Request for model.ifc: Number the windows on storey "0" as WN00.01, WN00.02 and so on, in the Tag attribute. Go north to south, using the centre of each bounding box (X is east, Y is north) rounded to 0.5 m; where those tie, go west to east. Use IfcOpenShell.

First a look at what the model holds.

```python
import ifcopenshell
import ifcopenshell.util.element
import ifcopenshell.util.placement

model = ifcopenshell.open("model.ifc")
print(model.schema)
storey = next(s for s in model.by_type("IfcBuildingStorey") if s.Name == "0")
windows = [e for e in ifcopenshell.util.element.get_decomposition(storey) if e.is_a("IfcWindow")]
for e in sorted(windows, key=lambda e: e.id()):
    origin = ifcopenshell.util.placement.get_local_placement(e.ObjectPlacement)[:3, 3]
    print(e.id(), e.Tag, e.Name, origin.round(2) + 0.0, sep=" | ")
```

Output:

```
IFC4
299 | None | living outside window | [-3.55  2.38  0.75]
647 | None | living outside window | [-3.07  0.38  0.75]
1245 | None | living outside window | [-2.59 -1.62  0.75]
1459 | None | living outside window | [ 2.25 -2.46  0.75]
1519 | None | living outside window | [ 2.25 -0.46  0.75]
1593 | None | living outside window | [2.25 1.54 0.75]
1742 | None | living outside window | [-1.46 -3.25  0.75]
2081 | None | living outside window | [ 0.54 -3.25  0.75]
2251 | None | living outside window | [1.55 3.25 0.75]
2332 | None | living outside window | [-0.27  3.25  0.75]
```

```python
import ifcopenshell
import ifcopenshell.geom
import ifcopenshell.util.element
import ifcopenshell.util.shape

model = ifcopenshell.open("model.ifc")
settings = ifcopenshell.geom.settings()
settings.set("use-world-coords", True)


def centre(element):
    shape = ifcopenshell.geom.create_shape(settings, element)
    return ifcopenshell.util.shape.get_bbox_centroid(shape.geometry)


storey = next(s for s in model.by_type("IfcBuildingStorey") if s.Name == "0")
windows = [e for e in ifcopenshell.util.element.get_decomposition(storey) if e.is_a("IfcWindow")]

# Insertion points can sit at a corner or the storey origin, so sort by the geometry (in metres).
centres = {e: centre(e) for e in windows}
windows.sort(key=lambda e: (-round(centres[e][1] / 0.5), centres[e][0]))

for i, e in enumerate(windows, start=1):
    number = f"WN00.{i:02d}"
    e.Tag = number
    print(e.id(), number)

model.write("model-out.ifc")
```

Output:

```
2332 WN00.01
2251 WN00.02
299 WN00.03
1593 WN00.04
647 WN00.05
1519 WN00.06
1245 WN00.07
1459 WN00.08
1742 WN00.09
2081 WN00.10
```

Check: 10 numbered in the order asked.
